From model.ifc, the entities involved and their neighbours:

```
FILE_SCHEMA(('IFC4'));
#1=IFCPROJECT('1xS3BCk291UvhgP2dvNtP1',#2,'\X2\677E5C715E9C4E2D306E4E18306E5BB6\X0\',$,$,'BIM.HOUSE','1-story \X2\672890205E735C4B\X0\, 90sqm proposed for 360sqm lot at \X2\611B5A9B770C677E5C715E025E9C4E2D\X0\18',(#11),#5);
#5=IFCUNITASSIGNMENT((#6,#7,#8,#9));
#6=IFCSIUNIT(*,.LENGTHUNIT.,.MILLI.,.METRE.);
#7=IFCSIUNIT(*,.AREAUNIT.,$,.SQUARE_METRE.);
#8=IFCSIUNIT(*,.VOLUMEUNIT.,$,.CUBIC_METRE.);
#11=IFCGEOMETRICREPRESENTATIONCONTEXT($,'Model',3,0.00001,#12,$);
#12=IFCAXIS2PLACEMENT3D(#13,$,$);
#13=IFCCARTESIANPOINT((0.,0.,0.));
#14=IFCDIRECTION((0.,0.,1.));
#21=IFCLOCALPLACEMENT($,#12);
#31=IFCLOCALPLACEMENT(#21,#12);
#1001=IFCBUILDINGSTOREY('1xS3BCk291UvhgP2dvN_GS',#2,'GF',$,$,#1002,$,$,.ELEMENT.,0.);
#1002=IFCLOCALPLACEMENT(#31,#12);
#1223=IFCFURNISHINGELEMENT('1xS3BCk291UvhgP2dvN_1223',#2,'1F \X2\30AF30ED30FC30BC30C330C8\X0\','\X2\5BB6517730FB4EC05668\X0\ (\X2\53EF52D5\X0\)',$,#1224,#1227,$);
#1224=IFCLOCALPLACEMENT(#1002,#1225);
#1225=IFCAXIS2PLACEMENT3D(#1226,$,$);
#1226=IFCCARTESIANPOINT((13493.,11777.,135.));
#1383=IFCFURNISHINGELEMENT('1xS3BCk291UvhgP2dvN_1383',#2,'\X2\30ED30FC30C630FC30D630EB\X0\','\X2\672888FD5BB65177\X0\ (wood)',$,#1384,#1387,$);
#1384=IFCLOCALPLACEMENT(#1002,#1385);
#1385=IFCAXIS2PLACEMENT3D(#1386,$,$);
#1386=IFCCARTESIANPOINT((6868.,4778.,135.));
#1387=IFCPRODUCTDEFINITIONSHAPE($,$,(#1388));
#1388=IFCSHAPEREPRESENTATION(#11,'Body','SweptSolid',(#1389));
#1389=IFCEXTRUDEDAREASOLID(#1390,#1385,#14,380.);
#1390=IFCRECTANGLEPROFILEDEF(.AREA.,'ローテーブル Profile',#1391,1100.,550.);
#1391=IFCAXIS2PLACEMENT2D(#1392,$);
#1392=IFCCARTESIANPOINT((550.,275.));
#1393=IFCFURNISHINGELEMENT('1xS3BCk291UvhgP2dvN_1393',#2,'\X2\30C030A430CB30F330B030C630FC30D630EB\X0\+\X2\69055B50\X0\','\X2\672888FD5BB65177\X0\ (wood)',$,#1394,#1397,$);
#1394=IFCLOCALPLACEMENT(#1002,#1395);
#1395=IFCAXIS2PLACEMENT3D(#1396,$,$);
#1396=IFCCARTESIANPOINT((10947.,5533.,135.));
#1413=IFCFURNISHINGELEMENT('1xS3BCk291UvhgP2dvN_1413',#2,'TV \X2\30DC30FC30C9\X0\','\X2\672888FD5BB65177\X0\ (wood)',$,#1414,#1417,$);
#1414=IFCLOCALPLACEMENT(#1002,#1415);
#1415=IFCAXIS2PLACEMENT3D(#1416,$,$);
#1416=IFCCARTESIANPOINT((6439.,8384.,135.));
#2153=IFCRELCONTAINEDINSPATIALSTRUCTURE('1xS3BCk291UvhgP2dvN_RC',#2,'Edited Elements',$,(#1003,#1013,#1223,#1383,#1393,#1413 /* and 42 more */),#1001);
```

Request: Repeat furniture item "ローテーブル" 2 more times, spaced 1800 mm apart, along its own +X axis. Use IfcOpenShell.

```python
import ifcopenshell
import ifcopenshell.api.geometry
import ifcopenshell.api.root
import ifcopenshell.util.element
import ifcopenshell.util.placement
import ifcopenshell.util.unit

model = ifcopenshell.open("model.ifc")
unit_scale = ifcopenshell.util.unit.calculate_unit_scale(model)


def reuse_history(source, copy):
    """copy_class also copies each property set's owner history, people and application; keep the originals."""
    for rel in copy.IsDefinedBy:
        if rel.is_a("IfcRelDefinesByProperties") and (history := rel.RelatingPropertyDefinition.OwnerHistory):
            rel.RelatingPropertyDefinition.OwnerHistory = source.OwnerHistory
            ifcopenshell.util.element.remove_deep2(model, history)


source = model.by_id(1383)
base = ifcopenshell.util.placement.get_local_placement(source.ObjectPlacement)
step = base[:3, 0] * 1.8 / unit_scale

for i in range(1, 3):
    copy = ifcopenshell.api.root.copy_class(model, product=source)
    copy.Representation = ifcopenshell.util.element.copy_deep(
        model, source.Representation, exclude=["IfcGeometricRepresentationContext", "IfcRepresentationMap"]
    )
    reuse_history(source, copy)
    matrix = base.copy()
    matrix[:3, 3] += i * step
    print("added at", matrix[:3, 3].round(3) + 0.0)
    ifcopenshell.api.geometry.edit_object_placement(model, product=copy, matrix=matrix, is_si=False)

model.write("model-out.ifc")
```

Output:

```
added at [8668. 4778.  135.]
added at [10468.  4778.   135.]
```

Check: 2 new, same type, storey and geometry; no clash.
